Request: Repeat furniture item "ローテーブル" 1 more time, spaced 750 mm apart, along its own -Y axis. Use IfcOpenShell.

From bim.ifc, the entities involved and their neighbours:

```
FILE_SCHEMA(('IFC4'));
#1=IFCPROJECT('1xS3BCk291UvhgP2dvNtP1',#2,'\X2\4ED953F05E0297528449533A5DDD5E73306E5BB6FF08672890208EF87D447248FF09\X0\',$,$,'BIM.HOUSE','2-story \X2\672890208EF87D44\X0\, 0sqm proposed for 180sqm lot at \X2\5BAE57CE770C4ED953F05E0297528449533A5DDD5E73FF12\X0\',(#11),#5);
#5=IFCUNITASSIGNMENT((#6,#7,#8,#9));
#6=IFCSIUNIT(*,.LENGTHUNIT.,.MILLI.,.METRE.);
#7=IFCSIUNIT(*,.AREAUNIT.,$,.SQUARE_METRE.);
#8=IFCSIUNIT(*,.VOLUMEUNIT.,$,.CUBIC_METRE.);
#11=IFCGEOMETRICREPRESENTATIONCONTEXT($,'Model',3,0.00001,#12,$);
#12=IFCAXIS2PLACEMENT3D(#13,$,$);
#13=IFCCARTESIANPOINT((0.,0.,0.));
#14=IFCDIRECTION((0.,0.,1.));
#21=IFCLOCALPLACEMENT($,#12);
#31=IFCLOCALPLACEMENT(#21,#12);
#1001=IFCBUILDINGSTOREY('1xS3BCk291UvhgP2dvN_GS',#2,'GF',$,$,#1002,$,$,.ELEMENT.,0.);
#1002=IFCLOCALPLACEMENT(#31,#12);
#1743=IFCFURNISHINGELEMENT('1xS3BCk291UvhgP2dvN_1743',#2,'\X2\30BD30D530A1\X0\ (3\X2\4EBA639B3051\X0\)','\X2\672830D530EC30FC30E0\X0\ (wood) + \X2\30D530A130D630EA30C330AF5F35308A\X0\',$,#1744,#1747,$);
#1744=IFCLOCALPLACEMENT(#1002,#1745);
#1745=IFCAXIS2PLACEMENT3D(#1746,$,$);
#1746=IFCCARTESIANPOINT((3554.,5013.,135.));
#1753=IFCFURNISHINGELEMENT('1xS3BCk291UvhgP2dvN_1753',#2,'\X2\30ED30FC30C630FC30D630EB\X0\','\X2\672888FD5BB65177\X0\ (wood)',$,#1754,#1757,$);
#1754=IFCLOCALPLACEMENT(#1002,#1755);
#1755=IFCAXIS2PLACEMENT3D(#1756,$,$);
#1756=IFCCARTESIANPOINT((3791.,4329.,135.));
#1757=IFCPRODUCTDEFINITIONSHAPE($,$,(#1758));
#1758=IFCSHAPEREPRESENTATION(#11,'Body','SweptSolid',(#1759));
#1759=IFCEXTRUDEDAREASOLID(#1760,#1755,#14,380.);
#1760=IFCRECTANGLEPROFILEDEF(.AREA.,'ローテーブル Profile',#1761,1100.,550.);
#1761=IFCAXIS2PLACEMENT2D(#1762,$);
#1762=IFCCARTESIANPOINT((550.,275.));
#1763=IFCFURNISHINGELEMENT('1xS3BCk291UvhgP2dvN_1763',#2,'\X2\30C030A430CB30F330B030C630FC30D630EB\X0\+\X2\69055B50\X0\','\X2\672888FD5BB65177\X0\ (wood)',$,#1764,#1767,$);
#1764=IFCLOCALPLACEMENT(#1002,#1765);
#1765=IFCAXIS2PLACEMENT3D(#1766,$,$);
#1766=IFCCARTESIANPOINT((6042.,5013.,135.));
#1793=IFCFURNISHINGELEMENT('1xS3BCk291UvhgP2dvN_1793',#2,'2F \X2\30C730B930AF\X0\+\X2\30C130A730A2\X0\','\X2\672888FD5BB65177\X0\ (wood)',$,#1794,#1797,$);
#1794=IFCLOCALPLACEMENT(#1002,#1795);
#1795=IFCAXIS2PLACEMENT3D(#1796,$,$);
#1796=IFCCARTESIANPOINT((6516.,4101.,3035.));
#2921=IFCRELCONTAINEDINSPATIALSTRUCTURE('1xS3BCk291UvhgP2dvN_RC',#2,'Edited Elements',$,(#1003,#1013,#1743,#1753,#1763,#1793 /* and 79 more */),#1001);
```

```python
import ifcopenshell
import ifcopenshell.api.geometry
import ifcopenshell.api.root
import ifcopenshell.util.element
import ifcopenshell.util.placement
import ifcopenshell.util.unit

model = ifcopenshell.open("bim.ifc")
unit_scale = ifcopenshell.util.unit.calculate_unit_scale(model)


def reuse_history(source, copy):
    """copy_class also copies each property set's owner history, people and application; keep the originals."""
    for rel in copy.IsDefinedBy:
        if rel.is_a("IfcRelDefinesByProperties") and (history := rel.RelatingPropertyDefinition.OwnerHistory):
            rel.RelatingPropertyDefinition.OwnerHistory = source.OwnerHistory
            ifcopenshell.util.element.remove_deep2(model, history)


source = model.by_guid("1xS3BCk291UvhgP2dvN_1753")
base = ifcopenshell.util.placement.get_local_placement(source.ObjectPlacement)
step = -base[:3, 1] * 0.75 / unit_scale

for i in range(1, 2):
    copy = ifcopenshell.api.root.copy_class(model, product=source)
    copy.Representation = ifcopenshell.util.element.copy_deep(
        model, source.Representation, exclude=["IfcGeometricRepresentationContext", "IfcRepresentationMap"]
    )
    reuse_history(source, copy)
    matrix = base.copy()
    matrix[:3, 3] += i * step
    print("added at", matrix[:3, 3].round(3) + 0.0)
    ifcopenshell.api.geometry.edit_object_placement(model, product=copy, matrix=matrix, is_si=False)

model.write("bim_updated.ifc")
```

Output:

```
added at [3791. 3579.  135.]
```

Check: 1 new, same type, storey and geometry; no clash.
